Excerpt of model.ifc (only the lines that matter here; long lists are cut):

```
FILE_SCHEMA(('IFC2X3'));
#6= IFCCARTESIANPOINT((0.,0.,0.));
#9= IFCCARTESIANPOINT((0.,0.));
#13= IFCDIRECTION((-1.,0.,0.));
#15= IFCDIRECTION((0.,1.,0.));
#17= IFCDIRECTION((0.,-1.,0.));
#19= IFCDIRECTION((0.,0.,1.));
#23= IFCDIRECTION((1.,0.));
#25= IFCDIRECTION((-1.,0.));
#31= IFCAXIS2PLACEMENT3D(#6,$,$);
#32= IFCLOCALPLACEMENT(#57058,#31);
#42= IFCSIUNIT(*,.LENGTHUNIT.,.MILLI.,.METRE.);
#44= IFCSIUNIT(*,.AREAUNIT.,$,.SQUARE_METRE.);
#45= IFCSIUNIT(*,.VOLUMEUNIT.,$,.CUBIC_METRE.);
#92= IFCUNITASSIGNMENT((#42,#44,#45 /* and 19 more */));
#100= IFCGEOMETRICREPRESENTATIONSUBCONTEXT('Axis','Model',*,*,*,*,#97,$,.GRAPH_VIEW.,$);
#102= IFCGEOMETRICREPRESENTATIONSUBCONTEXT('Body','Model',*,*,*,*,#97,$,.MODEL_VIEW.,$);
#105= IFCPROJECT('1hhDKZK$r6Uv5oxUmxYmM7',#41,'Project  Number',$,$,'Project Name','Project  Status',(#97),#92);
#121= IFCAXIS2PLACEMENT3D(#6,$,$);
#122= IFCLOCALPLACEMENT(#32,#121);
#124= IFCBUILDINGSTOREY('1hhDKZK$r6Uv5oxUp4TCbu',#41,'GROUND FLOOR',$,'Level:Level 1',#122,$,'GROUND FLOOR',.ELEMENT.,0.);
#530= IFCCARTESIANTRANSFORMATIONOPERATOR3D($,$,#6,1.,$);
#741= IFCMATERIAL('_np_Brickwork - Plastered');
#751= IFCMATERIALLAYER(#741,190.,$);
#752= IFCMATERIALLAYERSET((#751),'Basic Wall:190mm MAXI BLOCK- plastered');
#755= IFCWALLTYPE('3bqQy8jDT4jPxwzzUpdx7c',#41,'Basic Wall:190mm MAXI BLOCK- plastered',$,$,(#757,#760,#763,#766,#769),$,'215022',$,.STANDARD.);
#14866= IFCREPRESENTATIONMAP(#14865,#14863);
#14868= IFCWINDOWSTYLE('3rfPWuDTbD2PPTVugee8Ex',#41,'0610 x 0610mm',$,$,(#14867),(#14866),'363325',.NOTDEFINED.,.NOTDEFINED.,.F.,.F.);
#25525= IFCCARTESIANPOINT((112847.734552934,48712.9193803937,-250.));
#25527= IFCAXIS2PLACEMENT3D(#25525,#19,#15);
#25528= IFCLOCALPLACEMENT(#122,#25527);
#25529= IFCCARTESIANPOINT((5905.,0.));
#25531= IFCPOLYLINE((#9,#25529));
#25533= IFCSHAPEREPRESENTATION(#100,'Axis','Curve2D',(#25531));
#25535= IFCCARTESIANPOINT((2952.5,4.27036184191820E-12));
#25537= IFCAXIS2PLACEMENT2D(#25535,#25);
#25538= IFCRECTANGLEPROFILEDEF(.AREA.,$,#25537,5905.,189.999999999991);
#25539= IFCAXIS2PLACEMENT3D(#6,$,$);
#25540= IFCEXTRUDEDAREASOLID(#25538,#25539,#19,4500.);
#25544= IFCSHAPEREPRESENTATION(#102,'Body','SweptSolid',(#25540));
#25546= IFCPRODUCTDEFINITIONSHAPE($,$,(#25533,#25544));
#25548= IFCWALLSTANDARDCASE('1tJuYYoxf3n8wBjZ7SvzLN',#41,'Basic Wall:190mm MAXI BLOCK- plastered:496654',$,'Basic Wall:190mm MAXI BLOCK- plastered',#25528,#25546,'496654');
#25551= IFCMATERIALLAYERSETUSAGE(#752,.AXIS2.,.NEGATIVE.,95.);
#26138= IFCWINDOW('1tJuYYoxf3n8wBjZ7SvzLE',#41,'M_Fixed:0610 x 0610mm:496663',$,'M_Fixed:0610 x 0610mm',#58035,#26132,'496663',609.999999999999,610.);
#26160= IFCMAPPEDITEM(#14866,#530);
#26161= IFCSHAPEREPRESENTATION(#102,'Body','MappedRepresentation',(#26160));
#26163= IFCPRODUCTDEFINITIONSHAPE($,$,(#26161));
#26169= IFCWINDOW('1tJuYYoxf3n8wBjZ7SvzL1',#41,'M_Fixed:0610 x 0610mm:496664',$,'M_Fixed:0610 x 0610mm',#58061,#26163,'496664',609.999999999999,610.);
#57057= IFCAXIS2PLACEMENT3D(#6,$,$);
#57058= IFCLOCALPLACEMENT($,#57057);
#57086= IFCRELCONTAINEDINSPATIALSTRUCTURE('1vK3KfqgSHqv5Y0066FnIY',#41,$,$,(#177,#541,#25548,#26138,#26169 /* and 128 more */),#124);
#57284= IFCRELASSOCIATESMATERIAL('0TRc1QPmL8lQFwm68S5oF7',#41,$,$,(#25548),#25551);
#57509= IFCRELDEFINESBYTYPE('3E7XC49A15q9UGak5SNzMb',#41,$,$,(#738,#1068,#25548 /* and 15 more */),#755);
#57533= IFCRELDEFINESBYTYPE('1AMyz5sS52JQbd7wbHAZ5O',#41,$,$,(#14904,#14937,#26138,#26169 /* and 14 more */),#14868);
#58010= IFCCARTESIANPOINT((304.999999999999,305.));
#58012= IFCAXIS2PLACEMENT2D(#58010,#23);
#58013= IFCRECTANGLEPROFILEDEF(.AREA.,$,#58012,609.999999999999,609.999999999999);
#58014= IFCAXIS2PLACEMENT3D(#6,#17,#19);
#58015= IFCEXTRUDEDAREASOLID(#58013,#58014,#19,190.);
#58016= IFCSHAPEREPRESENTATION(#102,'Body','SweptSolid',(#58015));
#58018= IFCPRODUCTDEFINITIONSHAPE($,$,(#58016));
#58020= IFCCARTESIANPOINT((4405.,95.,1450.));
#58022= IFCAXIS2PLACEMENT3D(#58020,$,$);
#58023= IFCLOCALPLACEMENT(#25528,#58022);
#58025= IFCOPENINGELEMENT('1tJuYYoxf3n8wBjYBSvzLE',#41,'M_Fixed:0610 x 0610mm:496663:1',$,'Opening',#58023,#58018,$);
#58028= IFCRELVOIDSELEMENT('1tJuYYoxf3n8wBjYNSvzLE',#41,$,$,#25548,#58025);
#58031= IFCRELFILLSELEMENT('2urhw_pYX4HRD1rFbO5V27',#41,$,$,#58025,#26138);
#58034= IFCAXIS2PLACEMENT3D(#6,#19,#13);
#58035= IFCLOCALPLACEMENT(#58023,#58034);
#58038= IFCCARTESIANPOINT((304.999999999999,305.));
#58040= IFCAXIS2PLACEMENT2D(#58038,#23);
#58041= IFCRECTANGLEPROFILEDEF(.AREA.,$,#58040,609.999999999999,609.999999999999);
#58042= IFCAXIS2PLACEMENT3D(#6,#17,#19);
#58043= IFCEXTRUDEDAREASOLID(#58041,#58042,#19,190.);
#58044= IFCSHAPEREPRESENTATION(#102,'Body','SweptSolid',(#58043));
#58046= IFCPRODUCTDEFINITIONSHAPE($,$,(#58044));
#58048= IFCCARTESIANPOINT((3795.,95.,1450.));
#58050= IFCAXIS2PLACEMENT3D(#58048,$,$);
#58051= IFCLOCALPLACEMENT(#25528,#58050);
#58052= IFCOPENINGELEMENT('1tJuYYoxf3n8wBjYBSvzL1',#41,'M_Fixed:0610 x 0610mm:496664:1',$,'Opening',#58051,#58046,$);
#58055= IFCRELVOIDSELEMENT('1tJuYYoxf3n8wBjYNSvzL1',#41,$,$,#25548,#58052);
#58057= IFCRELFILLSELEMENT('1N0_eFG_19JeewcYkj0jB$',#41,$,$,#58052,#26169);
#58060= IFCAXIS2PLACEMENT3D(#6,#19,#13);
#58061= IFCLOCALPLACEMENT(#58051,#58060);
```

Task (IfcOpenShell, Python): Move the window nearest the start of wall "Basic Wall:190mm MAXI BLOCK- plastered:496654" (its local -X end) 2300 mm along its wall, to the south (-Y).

```python
import ifcopenshell
import ifcopenshell.api.geometry
import ifcopenshell.util.placement

model = ifcopenshell.open("model.ifc")

window = model.by_guid("1tJuYYoxf3n8wBjZ7SvzL1")
opening = window.FillsVoids[0].RelatingOpeningElement
wall = opening.VoidsElements[0].RelatingBuildingElement

wall_matrix = ifcopenshell.util.placement.get_local_placement(wall.ObjectPlacement)
shift = wall_matrix[:3, 0] * -2300.0
before = ifcopenshell.util.placement.get_local_placement(window.ObjectPlacement)[:3, 3].copy()

# The window is placed relative to its opening, so it follows when the opening moves.
matrix = ifcopenshell.util.placement.get_local_placement(opening.ObjectPlacement)
matrix[:3, 3] += shift
ifcopenshell.api.geometry.edit_object_placement(
    model, product=opening, matrix=matrix, is_si=False, should_transform_children=True
)

after = ifcopenshell.util.placement.get_local_placement(window.ObjectPlacement)[:3, 3]
print("window moved by", (after - before).round(3) + 0.0)

model.write("model_rev.ifc")
```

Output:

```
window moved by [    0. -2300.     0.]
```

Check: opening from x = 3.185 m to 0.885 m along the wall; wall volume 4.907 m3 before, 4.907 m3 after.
